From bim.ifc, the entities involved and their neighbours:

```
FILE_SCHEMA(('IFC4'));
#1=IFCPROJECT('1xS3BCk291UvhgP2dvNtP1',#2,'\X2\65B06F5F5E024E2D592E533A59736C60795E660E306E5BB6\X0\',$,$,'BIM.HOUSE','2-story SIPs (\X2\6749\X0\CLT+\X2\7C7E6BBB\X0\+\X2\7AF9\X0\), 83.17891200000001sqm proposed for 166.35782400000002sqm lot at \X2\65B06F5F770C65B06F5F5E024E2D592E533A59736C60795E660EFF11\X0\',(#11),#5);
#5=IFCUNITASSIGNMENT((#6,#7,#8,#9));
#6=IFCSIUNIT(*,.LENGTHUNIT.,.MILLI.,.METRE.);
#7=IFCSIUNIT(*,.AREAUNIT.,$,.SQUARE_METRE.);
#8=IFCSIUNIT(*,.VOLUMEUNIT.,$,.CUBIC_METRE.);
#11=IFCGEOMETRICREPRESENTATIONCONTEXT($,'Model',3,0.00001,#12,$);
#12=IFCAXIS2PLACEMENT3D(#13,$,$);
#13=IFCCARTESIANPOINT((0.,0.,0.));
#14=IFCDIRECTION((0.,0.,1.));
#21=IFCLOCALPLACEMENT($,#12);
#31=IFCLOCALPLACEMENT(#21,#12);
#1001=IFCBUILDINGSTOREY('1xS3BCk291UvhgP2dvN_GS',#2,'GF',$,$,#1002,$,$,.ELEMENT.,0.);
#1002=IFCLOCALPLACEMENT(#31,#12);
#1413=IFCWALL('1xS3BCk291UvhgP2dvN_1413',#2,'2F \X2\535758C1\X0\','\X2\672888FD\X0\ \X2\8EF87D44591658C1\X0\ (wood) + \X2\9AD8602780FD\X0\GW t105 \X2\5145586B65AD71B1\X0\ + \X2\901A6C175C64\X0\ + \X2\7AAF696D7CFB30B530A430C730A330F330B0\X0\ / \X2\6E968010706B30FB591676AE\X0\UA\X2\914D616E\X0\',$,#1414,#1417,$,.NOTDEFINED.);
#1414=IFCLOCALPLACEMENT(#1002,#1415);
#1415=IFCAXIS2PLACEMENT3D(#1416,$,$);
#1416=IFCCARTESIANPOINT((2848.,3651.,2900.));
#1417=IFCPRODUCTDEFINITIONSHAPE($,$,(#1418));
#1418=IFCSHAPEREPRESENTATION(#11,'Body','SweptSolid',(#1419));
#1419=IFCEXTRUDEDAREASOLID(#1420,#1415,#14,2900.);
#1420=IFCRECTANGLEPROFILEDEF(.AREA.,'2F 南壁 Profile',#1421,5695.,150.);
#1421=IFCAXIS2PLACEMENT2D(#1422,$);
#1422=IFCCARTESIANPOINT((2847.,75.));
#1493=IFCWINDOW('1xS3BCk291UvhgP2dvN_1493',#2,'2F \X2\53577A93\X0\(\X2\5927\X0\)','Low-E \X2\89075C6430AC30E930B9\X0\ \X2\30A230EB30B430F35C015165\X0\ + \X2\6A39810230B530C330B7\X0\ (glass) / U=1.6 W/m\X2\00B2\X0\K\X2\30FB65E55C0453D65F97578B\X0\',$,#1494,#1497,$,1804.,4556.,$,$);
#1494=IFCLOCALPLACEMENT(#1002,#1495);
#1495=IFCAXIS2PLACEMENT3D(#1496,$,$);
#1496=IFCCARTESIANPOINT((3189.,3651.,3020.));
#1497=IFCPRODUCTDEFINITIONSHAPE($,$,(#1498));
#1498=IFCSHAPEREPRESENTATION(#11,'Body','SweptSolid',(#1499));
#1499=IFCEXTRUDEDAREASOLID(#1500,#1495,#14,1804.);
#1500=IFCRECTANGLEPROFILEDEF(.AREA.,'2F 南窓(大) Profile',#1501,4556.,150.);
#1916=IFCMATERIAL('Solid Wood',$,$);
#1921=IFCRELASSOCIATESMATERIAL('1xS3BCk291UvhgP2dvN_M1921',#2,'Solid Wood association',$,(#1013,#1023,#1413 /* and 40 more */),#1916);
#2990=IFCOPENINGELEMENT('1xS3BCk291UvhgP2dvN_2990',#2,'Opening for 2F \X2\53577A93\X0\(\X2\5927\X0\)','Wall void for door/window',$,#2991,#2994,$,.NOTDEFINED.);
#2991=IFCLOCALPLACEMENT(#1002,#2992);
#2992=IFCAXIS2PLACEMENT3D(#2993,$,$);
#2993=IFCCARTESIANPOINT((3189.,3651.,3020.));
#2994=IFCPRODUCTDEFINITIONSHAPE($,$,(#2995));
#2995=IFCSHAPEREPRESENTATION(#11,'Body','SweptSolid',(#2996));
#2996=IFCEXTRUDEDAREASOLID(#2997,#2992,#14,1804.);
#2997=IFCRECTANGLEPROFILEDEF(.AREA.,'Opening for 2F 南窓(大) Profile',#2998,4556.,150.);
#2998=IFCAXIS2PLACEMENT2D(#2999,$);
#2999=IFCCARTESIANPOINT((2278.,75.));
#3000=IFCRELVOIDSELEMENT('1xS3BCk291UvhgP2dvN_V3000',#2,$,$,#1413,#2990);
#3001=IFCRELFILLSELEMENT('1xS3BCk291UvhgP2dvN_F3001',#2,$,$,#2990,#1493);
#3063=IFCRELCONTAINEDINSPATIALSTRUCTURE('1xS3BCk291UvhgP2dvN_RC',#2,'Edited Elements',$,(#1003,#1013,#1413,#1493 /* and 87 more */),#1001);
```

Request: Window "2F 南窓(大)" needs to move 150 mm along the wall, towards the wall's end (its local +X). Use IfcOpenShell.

```python
import ifcopenshell
import ifcopenshell.api.geometry
import ifcopenshell.util.placement
import ifcopenshell.util.unit

model = ifcopenshell.open("bim.ifc")
unit_scale = ifcopenshell.util.unit.calculate_unit_scale(model)

window = model.by_id(1493)
opening = window.FillsVoids[0].RelatingOpeningElement
wall = opening.VoidsElements[0].RelatingBuildingElement

wall_matrix = ifcopenshell.util.placement.get_local_placement(wall.ObjectPlacement)
shift = wall_matrix[:3, 0] * 0.15 / unit_scale
before = ifcopenshell.util.placement.get_local_placement(window.ObjectPlacement)[:3, 3].copy()

# The window is not placed relative to its opening, so move both.
for product in (opening, window):
    matrix = ifcopenshell.util.placement.get_local_placement(product.ObjectPlacement)
    matrix[:3, 3] += shift
    ifcopenshell.api.geometry.edit_object_placement(model, product=product, matrix=matrix, is_si=False)

after = ifcopenshell.util.placement.get_local_placement(window.ObjectPlacement)[:3, 3]
print("window moved by", (after - before).round(3) + 0.0)

model.write("bim-out.ifc")
```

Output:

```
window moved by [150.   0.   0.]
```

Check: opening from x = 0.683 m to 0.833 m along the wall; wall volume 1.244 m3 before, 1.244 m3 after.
